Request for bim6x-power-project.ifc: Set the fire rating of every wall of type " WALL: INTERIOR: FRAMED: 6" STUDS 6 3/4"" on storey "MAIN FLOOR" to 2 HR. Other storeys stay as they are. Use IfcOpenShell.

First a look at what the model holds.

```python
import ifcopenshell
import ifcopenshell.util.element

model = ifcopenshell.open("bim6x-power-project.ifc")
print(model.schema)
storey = next(s for s in model.by_type("IfcBuildingStorey") if s.Name == "MAIN FLOOR")
walls = [e for e in ifcopenshell.util.element.get_decomposition(storey) if e.is_a("IfcWall")]
seen = {}
for e in walls:
    element_type = ifcopenshell.util.element.get_type(e)
    key = (element_type.Name if element_type != e and element_type else None, ifcopenshell.util.element.get_pset(e, "Pset_WallCommon", "FireRating"))
    seen[key] = seen.get(key, 0) + 1
for (name, value), count in sorted(seen.items(), key=str):
    print(count, "x", name, "|", value)
```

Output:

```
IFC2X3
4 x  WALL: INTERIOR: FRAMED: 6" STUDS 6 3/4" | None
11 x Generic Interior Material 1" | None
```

```python
import ifcopenshell
import ifcopenshell.api.pset
import ifcopenshell.util.element

model = ifcopenshell.open("bim6x-power-project.ifc")

storey = next(s for s in model.by_type("IfcBuildingStorey") if s.Name == "MAIN FLOOR")
walls = [e for e in ifcopenshell.util.element.get_decomposition(storey) if e.is_a("IfcWall")]

count = 0
for e in walls:
    element_type = ifcopenshell.util.element.get_type(e)
    if element_type in (None, e) or element_type.Name != ' WALL: INTERIOR: FRAMED: 6" STUDS 6 3/4"':
        continue
    # add_pset returns the element's existing set when there is one.
    pset = ifcopenshell.api.pset.add_pset(model, product=e, name="Pset_WallCommon")
    ifcopenshell.api.pset.edit_pset(model, pset=pset, properties={"FireRating": "2 HR"})
    count += 1

print(count, "walls updated")

model.write("bim6x-power-project-out.ifc")
```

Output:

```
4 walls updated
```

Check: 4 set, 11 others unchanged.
